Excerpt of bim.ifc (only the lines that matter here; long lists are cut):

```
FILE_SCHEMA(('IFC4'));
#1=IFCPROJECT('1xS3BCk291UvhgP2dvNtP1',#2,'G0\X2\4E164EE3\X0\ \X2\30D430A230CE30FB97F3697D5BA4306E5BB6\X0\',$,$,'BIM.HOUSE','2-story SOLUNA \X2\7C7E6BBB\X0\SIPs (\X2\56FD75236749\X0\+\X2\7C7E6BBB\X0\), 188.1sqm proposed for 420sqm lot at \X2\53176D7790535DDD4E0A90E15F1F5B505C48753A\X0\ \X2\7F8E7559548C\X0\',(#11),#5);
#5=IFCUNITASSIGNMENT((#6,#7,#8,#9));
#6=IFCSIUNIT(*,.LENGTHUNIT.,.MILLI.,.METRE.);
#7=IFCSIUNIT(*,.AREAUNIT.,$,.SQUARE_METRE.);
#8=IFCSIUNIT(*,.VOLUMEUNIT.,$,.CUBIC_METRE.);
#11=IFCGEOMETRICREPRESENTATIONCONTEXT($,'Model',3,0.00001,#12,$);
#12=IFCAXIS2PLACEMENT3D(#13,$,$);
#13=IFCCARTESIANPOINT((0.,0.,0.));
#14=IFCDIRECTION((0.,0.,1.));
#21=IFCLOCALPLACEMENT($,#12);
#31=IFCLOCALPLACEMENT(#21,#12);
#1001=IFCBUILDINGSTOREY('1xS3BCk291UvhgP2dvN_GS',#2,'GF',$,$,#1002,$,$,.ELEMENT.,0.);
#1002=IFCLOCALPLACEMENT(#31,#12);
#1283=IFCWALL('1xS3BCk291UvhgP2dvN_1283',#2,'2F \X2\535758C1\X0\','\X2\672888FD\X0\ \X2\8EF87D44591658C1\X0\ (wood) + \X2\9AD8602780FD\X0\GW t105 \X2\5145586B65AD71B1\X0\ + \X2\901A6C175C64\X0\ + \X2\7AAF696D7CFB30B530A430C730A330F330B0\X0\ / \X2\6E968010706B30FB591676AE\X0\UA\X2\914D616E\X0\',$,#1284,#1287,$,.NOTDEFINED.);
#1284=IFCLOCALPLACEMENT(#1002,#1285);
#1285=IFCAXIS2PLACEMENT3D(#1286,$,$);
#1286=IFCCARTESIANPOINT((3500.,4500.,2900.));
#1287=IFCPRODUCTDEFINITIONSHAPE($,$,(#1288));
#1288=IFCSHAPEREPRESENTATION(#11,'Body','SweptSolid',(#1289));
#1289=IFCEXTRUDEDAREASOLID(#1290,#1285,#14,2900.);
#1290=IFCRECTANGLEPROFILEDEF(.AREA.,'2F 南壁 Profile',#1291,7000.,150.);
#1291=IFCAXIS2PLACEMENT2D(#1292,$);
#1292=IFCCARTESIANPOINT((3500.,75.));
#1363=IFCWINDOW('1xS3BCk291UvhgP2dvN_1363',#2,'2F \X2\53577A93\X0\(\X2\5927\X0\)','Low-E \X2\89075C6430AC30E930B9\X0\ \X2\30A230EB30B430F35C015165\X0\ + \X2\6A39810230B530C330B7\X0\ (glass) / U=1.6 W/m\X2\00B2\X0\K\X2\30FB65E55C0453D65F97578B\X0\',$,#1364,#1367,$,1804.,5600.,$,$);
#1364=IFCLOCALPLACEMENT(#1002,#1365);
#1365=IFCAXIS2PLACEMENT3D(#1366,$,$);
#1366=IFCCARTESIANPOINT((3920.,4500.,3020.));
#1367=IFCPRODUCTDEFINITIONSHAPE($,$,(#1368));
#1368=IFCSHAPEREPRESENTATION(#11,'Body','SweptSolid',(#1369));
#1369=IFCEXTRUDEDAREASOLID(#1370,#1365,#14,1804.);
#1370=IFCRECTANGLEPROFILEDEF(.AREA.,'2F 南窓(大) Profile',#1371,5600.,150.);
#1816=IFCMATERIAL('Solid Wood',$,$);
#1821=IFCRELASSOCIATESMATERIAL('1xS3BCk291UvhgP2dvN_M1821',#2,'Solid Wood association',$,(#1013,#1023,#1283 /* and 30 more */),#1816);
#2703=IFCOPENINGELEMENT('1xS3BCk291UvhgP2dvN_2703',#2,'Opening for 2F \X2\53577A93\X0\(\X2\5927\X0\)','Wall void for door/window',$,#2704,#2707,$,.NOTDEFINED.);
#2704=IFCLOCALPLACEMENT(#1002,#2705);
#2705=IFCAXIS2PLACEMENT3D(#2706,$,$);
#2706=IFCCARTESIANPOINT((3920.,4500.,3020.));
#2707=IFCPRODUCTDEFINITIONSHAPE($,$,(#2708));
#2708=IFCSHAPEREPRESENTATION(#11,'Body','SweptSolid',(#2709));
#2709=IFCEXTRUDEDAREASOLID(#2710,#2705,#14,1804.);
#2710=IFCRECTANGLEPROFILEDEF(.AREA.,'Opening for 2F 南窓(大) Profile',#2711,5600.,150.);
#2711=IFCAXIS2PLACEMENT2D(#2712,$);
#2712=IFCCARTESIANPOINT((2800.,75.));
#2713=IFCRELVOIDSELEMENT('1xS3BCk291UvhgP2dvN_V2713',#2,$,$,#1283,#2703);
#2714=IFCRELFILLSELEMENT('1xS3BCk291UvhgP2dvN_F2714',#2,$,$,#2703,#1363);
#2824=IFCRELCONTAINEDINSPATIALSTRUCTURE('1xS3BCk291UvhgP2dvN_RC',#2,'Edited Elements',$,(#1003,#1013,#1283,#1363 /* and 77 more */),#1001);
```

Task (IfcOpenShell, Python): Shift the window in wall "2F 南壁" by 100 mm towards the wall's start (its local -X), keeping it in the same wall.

```python
import ifcopenshell
import ifcopenshell.api.geometry
import ifcopenshell.util.placement

model = ifcopenshell.open("bim.ifc")

window = model.by_id(1363)
opening = window.FillsVoids[0].RelatingOpeningElement
wall = opening.VoidsElements[0].RelatingBuildingElement

wall_matrix = ifcopenshell.util.placement.get_local_placement(wall.ObjectPlacement)
shift = wall_matrix[:3, 0] * -100.0
before = ifcopenshell.util.placement.get_local_placement(window.ObjectPlacement)[:3, 3].copy()

# The window is not placed relative to its opening, so move both.
for product in (opening, window):
    matrix = ifcopenshell.util.placement.get_local_placement(product.ObjectPlacement)
    matrix[:3, 3] += shift
    ifcopenshell.api.geometry.edit_object_placement(model, product=product, matrix=matrix, is_si=False)

after = ifcopenshell.util.placement.get_local_placement(window.ObjectPlacement)[:3, 3]
print("window moved by", (after - before).round(3) + 0.0)

model.write("bim_updated.ifc")
```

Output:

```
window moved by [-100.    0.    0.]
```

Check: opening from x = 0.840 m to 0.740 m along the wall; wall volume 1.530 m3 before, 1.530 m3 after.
